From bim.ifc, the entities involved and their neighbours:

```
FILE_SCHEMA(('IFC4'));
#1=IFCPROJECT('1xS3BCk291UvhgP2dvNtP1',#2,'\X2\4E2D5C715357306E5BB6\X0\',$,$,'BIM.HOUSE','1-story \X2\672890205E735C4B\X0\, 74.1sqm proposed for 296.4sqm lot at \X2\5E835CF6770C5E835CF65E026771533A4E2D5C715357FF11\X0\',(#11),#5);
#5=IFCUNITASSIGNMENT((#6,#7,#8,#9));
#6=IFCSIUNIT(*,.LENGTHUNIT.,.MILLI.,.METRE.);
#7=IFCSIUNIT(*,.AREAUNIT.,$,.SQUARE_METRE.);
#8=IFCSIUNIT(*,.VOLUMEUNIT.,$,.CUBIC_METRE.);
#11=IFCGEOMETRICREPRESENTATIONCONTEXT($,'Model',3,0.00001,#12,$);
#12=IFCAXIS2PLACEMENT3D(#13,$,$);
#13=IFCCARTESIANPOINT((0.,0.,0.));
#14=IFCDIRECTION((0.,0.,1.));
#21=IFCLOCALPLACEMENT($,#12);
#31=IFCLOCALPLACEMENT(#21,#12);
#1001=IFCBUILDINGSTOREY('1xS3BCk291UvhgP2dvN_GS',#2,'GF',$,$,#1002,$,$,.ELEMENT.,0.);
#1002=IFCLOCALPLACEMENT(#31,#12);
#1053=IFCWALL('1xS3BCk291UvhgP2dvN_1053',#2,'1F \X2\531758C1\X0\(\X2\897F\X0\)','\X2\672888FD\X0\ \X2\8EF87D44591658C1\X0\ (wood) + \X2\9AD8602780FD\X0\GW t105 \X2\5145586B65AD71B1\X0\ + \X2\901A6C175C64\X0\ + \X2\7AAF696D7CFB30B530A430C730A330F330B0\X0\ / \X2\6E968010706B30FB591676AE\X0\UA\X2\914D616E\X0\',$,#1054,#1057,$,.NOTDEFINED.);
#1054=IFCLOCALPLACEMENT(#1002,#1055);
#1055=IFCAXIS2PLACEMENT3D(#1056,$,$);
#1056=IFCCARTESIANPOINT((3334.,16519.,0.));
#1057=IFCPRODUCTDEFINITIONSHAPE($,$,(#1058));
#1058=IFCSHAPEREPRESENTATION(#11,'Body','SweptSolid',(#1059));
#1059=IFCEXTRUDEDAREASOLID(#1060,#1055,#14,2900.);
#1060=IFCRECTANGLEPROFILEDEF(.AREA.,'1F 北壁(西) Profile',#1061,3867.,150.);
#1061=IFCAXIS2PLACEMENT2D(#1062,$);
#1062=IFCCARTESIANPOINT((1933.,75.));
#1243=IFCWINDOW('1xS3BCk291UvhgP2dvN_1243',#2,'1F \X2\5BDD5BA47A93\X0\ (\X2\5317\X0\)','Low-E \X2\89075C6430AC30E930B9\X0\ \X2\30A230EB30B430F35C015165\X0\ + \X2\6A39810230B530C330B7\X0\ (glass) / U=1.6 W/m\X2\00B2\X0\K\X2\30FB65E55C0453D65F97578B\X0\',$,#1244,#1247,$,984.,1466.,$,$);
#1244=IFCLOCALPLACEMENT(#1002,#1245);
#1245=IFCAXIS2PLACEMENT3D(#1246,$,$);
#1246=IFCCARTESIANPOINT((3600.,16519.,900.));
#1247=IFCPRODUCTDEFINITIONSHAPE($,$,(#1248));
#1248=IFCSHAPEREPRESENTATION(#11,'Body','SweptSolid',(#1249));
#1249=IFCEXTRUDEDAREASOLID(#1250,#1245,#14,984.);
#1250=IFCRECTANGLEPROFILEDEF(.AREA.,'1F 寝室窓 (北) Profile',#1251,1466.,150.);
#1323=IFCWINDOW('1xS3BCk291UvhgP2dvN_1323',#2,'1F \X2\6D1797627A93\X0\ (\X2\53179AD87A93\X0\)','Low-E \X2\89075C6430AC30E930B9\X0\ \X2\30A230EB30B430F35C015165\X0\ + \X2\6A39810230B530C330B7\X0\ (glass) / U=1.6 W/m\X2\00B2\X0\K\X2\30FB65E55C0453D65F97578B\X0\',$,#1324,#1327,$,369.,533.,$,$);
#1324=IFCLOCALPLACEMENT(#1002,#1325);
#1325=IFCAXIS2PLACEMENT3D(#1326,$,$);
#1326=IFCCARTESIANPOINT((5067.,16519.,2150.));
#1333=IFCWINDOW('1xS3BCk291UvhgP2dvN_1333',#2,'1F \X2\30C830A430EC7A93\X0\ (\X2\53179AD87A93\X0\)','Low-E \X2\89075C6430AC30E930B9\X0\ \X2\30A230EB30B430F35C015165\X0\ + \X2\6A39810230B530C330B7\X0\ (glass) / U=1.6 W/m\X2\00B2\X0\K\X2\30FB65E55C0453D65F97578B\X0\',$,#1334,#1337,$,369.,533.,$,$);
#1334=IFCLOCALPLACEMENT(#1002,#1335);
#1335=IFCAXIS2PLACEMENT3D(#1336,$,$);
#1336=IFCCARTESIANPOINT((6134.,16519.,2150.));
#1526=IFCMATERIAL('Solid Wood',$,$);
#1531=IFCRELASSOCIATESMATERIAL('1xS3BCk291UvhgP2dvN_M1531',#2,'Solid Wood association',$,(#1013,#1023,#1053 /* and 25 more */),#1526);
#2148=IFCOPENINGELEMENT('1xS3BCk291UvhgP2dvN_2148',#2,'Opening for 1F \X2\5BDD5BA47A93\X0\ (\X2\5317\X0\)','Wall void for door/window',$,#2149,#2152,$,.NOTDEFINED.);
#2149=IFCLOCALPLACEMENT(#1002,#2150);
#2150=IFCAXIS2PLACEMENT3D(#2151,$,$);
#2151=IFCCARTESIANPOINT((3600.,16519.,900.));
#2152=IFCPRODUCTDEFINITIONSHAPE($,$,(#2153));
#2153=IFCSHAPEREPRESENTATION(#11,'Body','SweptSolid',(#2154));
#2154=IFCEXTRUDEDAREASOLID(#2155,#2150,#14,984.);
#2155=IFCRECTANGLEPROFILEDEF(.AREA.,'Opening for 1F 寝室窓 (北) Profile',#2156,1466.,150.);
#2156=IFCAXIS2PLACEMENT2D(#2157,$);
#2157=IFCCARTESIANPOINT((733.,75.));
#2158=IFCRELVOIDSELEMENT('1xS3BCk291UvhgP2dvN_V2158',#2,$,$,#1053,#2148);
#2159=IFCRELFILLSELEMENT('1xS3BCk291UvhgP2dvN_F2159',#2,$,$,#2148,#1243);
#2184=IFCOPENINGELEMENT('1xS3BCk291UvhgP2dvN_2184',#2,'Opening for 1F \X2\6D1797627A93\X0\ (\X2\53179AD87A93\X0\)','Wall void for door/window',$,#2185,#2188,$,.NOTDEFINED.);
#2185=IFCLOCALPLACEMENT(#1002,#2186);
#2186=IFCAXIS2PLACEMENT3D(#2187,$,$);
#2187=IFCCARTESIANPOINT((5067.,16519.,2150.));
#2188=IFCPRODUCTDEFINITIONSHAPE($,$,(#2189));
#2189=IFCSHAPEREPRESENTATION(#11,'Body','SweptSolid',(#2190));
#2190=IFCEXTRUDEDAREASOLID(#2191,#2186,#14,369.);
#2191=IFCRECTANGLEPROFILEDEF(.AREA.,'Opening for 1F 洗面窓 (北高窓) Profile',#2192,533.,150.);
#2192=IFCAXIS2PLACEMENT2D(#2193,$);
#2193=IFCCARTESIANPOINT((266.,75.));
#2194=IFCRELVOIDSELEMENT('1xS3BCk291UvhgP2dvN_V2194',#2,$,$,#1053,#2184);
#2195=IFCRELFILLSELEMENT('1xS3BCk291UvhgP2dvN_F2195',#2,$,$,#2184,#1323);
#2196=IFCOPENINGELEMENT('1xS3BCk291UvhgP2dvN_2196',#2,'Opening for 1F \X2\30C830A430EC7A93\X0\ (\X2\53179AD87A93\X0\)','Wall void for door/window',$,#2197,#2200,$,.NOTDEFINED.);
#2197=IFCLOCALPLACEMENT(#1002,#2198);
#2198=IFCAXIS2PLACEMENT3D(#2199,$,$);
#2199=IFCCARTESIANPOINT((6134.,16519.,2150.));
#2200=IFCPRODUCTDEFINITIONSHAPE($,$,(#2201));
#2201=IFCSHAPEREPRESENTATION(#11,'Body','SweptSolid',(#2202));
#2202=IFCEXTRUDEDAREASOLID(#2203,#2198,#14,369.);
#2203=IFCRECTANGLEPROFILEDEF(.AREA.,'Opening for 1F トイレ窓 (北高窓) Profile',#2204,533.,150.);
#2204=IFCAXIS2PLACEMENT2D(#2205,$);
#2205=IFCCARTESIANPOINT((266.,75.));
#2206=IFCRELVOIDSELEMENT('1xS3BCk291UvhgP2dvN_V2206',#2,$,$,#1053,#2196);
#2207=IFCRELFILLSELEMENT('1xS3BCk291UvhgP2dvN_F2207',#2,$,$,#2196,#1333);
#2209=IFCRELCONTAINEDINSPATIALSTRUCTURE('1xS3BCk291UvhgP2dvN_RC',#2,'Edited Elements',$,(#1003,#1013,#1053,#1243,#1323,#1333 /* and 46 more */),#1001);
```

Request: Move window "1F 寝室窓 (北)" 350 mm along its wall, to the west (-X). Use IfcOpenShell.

```python
import ifcopenshell
import ifcopenshell.api.geometry
import ifcopenshell.util.placement
import ifcopenshell.util.unit

model = ifcopenshell.open("bim.ifc")
unit_scale = ifcopenshell.util.unit.calculate_unit_scale(model)

window = model.by_guid("1xS3BCk291UvhgP2dvN_1243")
opening = window.FillsVoids[0].RelatingOpeningElement
wall = opening.VoidsElements[0].RelatingBuildingElement

wall_matrix = ifcopenshell.util.placement.get_local_placement(wall.ObjectPlacement)
shift = wall_matrix[:3, 0] * -0.35 / unit_scale
before = ifcopenshell.util.placement.get_local_placement(window.ObjectPlacement)[:3, 3].copy()

# The window is not placed relative to its opening, so move both.
for product in (opening, window):
    matrix = ifcopenshell.util.placement.get_local_placement(product.ObjectPlacement)
    matrix[:3, 3] += shift
    ifcopenshell.api.geometry.edit_object_placement(model, product=product, matrix=matrix, is_si=False)

after = ifcopenshell.util.placement.get_local_placement(window.ObjectPlacement)[:3, 3]
print("window moved by", (after - before).round(3) + 0.0)

model.write("bim-out.ifc")
```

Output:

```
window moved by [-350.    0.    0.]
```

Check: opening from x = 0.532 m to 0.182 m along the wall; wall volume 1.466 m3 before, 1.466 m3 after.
